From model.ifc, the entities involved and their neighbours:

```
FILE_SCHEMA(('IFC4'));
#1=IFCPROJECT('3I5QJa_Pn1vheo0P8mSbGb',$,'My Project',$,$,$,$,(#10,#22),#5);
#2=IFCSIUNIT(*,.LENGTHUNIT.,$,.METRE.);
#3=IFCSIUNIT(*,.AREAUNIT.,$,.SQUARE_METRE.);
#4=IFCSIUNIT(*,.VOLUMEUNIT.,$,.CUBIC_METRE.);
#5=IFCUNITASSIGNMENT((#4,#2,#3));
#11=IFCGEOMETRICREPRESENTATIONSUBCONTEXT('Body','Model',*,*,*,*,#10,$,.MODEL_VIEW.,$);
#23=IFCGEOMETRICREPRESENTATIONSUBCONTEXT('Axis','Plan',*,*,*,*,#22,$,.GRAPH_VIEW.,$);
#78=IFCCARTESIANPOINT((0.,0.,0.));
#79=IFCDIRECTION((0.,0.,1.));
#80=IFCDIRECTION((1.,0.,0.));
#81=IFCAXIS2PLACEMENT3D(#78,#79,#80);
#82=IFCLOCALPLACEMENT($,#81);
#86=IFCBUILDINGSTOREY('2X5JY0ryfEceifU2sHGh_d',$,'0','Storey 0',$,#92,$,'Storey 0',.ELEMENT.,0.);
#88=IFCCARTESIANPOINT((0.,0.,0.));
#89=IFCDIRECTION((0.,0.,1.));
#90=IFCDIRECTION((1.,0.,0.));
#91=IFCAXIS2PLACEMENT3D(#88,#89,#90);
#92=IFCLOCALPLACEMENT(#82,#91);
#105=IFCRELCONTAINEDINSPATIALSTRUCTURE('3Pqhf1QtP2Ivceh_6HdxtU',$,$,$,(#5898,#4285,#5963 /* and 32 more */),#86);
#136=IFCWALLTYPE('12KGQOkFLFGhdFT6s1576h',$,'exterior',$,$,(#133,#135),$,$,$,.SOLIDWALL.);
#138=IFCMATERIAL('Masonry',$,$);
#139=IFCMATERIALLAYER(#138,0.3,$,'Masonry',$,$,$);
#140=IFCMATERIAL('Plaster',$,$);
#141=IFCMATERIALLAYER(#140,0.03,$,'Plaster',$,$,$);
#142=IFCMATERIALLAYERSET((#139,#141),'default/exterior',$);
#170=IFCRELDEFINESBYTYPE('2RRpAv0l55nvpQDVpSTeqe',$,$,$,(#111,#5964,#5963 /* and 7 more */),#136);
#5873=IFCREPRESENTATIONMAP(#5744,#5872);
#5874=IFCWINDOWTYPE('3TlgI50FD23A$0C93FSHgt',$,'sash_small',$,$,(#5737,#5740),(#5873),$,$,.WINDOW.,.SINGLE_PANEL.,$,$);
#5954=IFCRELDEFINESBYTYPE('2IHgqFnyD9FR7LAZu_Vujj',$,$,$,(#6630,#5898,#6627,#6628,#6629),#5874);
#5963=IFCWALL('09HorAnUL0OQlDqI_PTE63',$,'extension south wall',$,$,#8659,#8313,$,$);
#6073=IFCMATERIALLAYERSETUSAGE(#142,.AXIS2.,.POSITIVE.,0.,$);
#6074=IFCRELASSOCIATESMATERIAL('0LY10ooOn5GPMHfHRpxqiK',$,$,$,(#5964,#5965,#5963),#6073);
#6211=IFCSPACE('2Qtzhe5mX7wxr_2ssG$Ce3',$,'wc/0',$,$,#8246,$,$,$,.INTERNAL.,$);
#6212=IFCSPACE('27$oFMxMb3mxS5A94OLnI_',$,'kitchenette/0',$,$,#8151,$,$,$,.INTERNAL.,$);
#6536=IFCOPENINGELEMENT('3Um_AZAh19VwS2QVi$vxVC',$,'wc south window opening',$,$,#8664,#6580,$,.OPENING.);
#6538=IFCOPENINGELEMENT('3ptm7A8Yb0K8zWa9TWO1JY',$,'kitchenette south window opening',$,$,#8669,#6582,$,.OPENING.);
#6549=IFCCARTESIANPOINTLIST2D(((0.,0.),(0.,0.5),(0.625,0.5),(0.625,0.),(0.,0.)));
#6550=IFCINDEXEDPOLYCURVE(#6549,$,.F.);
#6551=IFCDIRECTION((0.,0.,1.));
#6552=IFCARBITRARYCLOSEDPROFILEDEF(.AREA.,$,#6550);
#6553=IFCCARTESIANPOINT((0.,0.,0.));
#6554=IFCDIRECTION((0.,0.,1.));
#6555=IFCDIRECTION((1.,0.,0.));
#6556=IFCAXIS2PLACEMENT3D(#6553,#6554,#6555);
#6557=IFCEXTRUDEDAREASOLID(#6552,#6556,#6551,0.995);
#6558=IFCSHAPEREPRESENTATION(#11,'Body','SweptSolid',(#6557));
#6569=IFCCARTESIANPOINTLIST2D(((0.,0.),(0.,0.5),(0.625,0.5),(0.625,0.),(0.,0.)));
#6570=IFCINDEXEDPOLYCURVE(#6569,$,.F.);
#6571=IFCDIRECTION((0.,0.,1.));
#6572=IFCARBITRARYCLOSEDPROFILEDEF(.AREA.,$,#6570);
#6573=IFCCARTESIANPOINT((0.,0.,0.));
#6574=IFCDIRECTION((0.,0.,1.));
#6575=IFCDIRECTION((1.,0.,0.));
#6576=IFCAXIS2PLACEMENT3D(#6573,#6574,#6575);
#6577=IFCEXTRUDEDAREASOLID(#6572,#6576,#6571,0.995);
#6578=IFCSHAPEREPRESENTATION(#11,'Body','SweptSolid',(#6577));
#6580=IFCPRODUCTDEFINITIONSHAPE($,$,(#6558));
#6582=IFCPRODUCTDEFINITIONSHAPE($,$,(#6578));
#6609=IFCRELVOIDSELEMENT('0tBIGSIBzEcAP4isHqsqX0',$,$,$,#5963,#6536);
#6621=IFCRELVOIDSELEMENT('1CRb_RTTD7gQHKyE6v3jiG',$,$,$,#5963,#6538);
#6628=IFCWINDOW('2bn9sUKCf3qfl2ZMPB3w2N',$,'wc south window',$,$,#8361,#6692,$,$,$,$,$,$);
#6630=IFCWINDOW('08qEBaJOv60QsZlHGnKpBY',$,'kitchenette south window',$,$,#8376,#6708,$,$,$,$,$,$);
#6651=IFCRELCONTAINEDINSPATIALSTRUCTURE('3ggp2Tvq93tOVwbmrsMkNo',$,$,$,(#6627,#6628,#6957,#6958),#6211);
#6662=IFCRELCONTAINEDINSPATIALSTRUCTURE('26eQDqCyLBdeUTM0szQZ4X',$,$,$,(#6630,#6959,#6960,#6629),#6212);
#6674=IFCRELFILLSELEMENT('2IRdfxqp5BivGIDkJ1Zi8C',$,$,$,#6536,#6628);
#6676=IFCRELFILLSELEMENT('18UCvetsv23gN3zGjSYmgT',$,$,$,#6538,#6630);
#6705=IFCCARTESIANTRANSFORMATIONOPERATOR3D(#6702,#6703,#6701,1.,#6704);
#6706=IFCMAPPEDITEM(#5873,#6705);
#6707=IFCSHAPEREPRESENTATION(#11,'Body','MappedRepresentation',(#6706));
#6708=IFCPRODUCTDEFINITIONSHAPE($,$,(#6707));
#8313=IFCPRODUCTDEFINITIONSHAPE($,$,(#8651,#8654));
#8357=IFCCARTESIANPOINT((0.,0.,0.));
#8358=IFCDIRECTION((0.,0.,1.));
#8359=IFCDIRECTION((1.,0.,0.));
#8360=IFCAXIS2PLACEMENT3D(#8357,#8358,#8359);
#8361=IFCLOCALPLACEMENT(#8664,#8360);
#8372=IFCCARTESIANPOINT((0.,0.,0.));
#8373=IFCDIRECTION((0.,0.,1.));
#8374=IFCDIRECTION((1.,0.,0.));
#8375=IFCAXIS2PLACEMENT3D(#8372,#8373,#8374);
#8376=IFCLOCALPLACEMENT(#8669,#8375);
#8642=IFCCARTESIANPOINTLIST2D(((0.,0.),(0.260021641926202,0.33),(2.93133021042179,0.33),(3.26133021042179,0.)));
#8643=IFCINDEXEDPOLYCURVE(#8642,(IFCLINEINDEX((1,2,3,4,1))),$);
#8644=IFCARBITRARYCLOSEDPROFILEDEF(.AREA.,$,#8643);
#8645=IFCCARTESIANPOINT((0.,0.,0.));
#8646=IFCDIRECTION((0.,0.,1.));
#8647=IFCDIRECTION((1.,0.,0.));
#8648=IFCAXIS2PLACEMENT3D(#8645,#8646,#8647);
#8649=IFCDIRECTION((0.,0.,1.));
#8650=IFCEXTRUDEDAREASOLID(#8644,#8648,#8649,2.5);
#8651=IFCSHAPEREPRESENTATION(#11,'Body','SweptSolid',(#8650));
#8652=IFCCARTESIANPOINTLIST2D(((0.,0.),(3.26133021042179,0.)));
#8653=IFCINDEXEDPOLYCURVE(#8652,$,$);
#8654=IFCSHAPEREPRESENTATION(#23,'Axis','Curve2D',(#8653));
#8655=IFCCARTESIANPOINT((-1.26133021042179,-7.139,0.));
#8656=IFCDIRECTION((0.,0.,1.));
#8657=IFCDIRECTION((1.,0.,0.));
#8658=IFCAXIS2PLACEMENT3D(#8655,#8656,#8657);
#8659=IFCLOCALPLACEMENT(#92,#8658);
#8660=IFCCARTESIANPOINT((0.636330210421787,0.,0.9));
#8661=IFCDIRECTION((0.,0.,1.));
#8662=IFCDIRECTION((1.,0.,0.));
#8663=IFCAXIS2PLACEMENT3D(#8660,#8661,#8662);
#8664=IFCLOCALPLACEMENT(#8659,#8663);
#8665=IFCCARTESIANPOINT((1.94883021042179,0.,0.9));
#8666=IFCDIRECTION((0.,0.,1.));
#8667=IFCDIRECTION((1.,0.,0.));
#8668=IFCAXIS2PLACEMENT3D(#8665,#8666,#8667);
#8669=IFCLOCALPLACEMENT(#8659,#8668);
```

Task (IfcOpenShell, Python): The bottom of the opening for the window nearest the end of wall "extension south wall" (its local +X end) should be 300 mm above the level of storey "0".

```python
import numpy as np
import ifcopenshell
import ifcopenshell.api.geometry
import ifcopenshell.geom
import ifcopenshell.util.element
import ifcopenshell.util.placement
import ifcopenshell.util.shape
import ifcopenshell.util.unit

model = ifcopenshell.open("model.ifc")
unit_scale = ifcopenshell.util.unit.calculate_unit_scale(model)

window = model.by_id(6630)
opening = window.FillsVoids[0].RelatingOpeningElement
storey = ifcopenshell.util.element.get_container(window, ifc_class="IfcBuildingStorey")
level = ifcopenshell.util.placement.get_local_placement(storey.ObjectPlacement)[2, 3]

# The opening's origin need not be at the sill, so measure its lowest point.
shape = ifcopenshell.geom.create_shape(ifcopenshell.geom.settings(), opening)
bottom = ifcopenshell.util.shape.get_shape_bottom_elevation(shape, shape.geometry) / unit_scale
dz = level + 0.3 / unit_scale - bottom

shift = np.array([0.0, 0.0, dz])
# The window is placed relative to its opening, so it follows when the opening moves.
matrix = ifcopenshell.util.placement.get_local_placement(opening.ObjectPlacement)
matrix[:3, 3] += shift
ifcopenshell.api.geometry.edit_object_placement(
    model, product=opening, matrix=matrix, is_si=False, should_transform_children=True
)

print(f"moved by {dz * unit_scale:+.3f} m")

model.write("model_updated.ifc")
```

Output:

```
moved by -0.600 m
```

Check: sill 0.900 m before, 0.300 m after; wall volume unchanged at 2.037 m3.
